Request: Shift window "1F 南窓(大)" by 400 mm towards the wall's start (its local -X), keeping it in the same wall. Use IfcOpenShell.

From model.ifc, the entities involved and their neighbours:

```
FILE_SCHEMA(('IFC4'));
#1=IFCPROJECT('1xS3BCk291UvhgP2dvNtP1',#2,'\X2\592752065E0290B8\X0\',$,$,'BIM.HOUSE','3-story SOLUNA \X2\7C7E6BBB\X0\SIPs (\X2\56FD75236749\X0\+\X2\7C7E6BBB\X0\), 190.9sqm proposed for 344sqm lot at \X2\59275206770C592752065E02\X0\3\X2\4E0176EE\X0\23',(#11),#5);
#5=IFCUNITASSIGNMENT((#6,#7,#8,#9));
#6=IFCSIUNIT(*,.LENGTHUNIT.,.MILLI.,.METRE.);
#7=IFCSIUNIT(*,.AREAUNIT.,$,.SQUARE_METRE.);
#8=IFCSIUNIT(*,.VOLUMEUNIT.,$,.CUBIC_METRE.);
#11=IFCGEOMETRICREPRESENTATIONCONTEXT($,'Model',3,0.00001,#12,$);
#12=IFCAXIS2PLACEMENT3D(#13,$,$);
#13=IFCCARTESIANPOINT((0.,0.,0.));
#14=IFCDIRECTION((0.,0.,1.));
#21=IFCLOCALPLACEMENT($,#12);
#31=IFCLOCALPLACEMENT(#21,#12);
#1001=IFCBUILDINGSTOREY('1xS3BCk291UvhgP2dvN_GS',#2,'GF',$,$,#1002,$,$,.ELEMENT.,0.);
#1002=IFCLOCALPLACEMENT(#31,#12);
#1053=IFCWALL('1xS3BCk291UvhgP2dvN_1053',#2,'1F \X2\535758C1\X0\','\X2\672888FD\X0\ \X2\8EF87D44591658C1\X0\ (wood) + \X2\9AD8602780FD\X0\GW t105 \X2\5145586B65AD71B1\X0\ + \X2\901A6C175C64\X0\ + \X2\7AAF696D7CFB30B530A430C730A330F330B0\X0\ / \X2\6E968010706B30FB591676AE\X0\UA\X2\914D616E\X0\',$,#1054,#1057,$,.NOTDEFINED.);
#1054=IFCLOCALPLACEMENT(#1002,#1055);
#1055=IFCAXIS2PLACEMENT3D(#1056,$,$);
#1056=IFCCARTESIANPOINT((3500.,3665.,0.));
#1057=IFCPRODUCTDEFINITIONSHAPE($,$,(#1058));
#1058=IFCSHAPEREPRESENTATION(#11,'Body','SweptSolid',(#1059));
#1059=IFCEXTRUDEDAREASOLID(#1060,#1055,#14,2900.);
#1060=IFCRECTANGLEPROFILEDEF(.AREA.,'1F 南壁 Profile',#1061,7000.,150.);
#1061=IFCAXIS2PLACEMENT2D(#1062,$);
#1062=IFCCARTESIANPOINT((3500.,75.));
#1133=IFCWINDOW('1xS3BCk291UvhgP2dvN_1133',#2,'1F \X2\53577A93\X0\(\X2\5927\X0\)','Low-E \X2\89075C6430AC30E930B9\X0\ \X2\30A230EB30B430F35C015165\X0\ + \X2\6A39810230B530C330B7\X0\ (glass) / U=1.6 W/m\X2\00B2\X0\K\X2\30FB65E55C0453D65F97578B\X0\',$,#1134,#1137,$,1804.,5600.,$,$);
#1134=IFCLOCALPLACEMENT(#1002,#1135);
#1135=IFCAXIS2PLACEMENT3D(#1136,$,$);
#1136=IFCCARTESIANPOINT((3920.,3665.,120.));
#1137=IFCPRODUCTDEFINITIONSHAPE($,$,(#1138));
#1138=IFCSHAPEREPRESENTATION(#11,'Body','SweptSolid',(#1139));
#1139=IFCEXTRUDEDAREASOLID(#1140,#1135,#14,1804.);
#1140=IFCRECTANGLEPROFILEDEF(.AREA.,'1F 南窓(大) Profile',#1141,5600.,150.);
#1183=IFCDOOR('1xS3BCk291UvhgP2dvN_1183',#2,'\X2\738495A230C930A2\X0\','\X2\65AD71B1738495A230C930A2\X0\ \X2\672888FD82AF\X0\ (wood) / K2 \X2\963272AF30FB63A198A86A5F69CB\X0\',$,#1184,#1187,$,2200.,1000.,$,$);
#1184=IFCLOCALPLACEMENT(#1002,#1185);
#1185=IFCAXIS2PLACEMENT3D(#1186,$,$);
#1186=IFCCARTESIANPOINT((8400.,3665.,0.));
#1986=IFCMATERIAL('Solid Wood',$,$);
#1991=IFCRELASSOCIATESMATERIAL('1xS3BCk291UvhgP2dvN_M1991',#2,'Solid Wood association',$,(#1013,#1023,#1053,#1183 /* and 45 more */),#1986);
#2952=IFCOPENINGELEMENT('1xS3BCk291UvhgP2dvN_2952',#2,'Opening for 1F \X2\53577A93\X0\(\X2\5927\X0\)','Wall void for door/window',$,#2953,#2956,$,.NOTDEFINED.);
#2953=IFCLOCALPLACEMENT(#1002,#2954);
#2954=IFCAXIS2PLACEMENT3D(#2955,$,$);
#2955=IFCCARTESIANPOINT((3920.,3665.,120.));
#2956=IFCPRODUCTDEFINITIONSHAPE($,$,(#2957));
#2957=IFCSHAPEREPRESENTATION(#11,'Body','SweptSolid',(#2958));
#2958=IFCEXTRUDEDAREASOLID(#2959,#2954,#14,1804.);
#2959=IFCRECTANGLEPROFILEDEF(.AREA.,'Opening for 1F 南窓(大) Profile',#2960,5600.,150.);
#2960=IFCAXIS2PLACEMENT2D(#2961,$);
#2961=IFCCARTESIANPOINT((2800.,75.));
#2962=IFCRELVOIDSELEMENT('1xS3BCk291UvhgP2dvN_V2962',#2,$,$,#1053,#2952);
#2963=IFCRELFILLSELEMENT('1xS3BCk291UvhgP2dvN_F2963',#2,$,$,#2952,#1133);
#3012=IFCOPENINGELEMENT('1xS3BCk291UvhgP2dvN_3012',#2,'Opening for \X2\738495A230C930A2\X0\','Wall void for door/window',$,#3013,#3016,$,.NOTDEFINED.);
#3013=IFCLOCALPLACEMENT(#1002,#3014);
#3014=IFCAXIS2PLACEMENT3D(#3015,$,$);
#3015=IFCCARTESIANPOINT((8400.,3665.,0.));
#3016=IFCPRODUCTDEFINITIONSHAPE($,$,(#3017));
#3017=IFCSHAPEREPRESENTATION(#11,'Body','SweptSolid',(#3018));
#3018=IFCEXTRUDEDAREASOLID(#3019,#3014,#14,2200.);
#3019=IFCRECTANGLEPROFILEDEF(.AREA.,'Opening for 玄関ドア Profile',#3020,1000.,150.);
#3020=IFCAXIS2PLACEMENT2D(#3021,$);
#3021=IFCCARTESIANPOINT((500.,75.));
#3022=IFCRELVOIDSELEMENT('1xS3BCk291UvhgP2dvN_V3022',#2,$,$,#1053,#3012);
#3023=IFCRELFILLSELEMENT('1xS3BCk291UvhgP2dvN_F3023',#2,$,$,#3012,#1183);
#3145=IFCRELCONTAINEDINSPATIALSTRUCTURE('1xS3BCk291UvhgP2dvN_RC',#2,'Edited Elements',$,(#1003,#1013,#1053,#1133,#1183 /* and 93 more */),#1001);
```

```python
import ifcopenshell
import ifcopenshell.api.geometry
import ifcopenshell.util.placement
import ifcopenshell.util.unit

model = ifcopenshell.open("model.ifc")
unit_scale = ifcopenshell.util.unit.calculate_unit_scale(model)

window = model.by_id(1133)
opening = window.FillsVoids[0].RelatingOpeningElement
wall = opening.VoidsElements[0].RelatingBuildingElement

wall_matrix = ifcopenshell.util.placement.get_local_placement(wall.ObjectPlacement)
shift = wall_matrix[:3, 0] * -0.4 / unit_scale
before = ifcopenshell.util.placement.get_local_placement(window.ObjectPlacement)[:3, 3].copy()

# The window is not placed relative to its opening, so move both.
for product in (opening, window):
    matrix = ifcopenshell.util.placement.get_local_placement(product.ObjectPlacement)
    matrix[:3, 3] += shift
    ifcopenshell.api.geometry.edit_object_placement(model, product=product, matrix=matrix, is_si=False)

after = ifcopenshell.util.placement.get_local_placement(window.ObjectPlacement)[:3, 3]
print("window moved by", (after - before).round(3) + 0.0)

model.write("model_v2.ifc")
```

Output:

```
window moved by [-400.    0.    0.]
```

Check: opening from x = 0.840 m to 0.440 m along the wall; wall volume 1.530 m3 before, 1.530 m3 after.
